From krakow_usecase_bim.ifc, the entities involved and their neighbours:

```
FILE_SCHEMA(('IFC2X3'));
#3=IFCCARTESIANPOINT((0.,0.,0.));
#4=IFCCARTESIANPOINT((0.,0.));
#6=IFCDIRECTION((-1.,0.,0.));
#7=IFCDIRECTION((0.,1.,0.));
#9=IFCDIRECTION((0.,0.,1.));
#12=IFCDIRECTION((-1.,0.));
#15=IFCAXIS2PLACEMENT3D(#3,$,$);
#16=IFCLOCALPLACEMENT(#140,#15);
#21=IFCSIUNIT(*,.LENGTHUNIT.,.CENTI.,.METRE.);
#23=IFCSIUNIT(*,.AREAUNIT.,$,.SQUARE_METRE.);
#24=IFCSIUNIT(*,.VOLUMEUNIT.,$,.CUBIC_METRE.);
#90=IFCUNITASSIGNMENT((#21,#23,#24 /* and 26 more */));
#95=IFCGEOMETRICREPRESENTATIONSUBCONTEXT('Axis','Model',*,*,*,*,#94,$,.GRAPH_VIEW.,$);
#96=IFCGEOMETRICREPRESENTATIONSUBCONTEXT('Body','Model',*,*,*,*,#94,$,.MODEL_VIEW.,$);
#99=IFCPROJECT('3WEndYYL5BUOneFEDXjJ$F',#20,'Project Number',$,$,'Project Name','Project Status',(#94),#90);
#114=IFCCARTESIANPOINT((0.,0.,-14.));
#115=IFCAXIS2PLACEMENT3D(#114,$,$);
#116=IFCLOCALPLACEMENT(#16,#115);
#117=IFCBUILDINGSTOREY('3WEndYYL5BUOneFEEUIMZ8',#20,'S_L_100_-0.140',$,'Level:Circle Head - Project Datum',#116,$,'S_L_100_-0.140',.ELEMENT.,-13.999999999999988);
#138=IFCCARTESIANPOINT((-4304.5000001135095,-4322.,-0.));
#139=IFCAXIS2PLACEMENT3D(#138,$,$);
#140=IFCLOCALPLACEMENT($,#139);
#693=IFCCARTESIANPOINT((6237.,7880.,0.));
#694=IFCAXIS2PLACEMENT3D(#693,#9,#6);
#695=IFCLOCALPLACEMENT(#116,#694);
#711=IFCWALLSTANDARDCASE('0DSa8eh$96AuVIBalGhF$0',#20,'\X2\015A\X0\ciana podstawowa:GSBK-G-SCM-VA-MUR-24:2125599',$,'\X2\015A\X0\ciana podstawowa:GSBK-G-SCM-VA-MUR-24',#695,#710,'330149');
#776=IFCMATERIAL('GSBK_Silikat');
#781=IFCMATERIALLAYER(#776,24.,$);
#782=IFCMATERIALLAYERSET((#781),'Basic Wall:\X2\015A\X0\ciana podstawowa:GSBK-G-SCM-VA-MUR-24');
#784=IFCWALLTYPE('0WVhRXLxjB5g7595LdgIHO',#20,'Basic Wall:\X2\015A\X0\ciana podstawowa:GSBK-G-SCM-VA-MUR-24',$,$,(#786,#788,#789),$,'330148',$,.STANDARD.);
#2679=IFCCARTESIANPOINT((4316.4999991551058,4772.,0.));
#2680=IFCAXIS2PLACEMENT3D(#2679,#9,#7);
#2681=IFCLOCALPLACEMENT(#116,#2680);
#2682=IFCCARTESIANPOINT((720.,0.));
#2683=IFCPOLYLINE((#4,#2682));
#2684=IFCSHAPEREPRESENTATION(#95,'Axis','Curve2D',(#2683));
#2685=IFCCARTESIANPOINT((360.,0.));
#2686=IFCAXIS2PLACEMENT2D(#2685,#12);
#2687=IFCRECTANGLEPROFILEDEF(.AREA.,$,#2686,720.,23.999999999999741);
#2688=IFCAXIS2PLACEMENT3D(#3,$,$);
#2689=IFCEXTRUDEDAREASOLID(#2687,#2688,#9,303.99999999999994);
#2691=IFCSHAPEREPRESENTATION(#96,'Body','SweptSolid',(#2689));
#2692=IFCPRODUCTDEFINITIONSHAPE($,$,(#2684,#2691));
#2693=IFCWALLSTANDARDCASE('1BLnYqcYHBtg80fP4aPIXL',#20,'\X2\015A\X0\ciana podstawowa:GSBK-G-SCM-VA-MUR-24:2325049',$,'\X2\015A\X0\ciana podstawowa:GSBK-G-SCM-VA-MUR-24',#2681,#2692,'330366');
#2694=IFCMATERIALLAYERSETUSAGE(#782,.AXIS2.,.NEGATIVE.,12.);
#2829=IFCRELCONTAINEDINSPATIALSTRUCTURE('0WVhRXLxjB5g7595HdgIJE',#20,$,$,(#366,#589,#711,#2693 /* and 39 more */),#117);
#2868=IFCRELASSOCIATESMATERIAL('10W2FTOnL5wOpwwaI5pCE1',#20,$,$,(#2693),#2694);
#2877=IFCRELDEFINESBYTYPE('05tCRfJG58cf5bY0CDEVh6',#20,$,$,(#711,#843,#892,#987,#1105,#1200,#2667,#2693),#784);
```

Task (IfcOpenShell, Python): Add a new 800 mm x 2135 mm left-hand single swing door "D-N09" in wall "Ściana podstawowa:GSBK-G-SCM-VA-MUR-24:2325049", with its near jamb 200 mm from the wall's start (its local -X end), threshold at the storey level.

```python
import numpy as np
import ifcopenshell
import ifcopenshell.api.feature
import ifcopenshell.api.geometry
import ifcopenshell.api.root
import ifcopenshell.api.spatial
import ifcopenshell.api.type
import ifcopenshell.geom
import ifcopenshell.util.element
import ifcopenshell.util.placement
import ifcopenshell.util.representation
import ifcopenshell.util.shape
import ifcopenshell.util.unit

model = ifcopenshell.open("krakow_usecase_bim.ifc")
unit_scale = ifcopenshell.util.unit.calculate_unit_scale(model)
settings = ifcopenshell.geom.settings()


def volume(element):
    """Net volume in cubic metres, openings subtracted."""
    shape = ifcopenshell.geom.create_shape(settings, element)
    return ifcopenshell.util.shape.get_volume(shape.geometry)


wall = model.by_guid("1BLnYqcYHBtg80fP4aPIXL")
storey = ifcopenshell.util.element.get_container(wall, ifc_class="IfcBuildingStorey")
context = ifcopenshell.util.representation.get_context(model, "Model", "Body", "MODEL_VIEW")
before = volume(wall)

width, height, from_end, sill = 0.8, 2.135, 0.2, 0.0  # metres

# The wall runs along its own X axis, and the end named is its -X end.
wall_shape = ifcopenshell.geom.create_shape(settings, wall)
x, y, z = ifcopenshell.util.shape.get_vertices(wall_shape.geometry).T
start = x.min() + from_end
face, thickness = float(y.min()), float(y.max() - y.min())
wall_matrix = ifcopenshell.util.placement.get_local_placement(wall.ObjectPlacement)
level = ifcopenshell.util.placement.get_local_placement(storey.ObjectPlacement)[2, 3]


def in_wall(x, y):
    """Placement at x, y metres in the wall's axes, at sill height."""
    matrix = wall_matrix.copy()
    matrix[:, 3] = wall_matrix @ np.array([x / unit_scale, y / unit_scale, 0.0, 1.0])
    matrix[2, 3] = level + sill / unit_scale
    return matrix


# Opening: a box that overshoots both wall faces by 50 mm.
opening = ifcopenshell.api.root.create_entity(model, ifc_class="IfcOpeningElement")
box = ifcopenshell.api.geometry.add_wall_representation(
    model, context=context, length=width, height=height, thickness=thickness + 0.1
)
ifcopenshell.api.geometry.assign_representation(model, product=opening, representation=box)
ifcopenshell.api.geometry.edit_object_placement(model, product=opening, matrix=in_wall(start, face - 0.05), is_si=False)
ifcopenshell.api.feature.add_feature(model, feature=opening, element=wall)

door = ifcopenshell.api.root.create_entity(model, ifc_class="IfcDoor", name="D-N09")
door.OverallWidth, door.OverallHeight = width / unit_scale, height / unit_scale
body = ifcopenshell.api.geometry.add_door_representation(
    model,
    context=context,
    overall_width=door.OverallWidth,
    overall_height=door.OverallHeight,
    operation_type="SINGLE_SWING_LEFT",
    lining_properties={"LiningDepth": thickness / unit_scale, "ThresholdDepth": thickness / unit_scale},
)
ifcopenshell.api.geometry.assign_representation(model, product=door, representation=body)
ifcopenshell.api.spatial.assign_container(model, products=[door], relating_structure=storey)
fills = ifcopenshell.api.feature.add_filling(model, opening=opening, element=door)
fills.OwnerHistory = door.OwnerHistory  # required in IFC2X3

# IFC2X3 keeps the operation on the door style.
style = ifcopenshell.api.root.create_entity(model, ifc_class="IfcDoorStyle", name="D-N09")
style.OperationType, style.ConstructionType = "SINGLE_SWING_LEFT", "NOTDEFINED"
style.ParameterTakesPrecedence = style.Sizeable = False
ifcopenshell.api.type.assign_type(model, related_objects=[door], relating_type=style)

# The lining spans the wall, so the door starts at the wall face.
ifcopenshell.api.geometry.edit_object_placement(model, product=door, matrix=in_wall(start, face), is_si=False)

after = volume(wall)

print(f"wall volume {before:.3f} -> {after:.3f} m3")

model.write("krakow_usecase_bim_v2.ifc")
```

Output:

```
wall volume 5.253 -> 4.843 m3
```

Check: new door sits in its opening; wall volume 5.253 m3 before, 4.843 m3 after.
